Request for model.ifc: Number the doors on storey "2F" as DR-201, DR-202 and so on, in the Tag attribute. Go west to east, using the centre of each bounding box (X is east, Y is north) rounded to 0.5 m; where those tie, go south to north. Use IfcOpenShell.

First a look at what the model holds.

```python
import ifcopenshell
import ifcopenshell.util.element
import ifcopenshell.util.placement

model = ifcopenshell.open("model.ifc")
print(model.schema)
storey = next(s for s in model.by_type("IfcBuildingStorey") if s.Name == "2F")
doors = [e for e in ifcopenshell.util.element.get_decomposition(storey) if e.is_a("IfcDoor")]
for e in sorted(doors, key=lambda e: e.id()):
    origin = ifcopenshell.util.placement.get_local_placement(e.ObjectPlacement)[:3, 3]
    print(e.id(), e.Tag, e.Name, origin.round(2) + 0.0, sep=" | ")
```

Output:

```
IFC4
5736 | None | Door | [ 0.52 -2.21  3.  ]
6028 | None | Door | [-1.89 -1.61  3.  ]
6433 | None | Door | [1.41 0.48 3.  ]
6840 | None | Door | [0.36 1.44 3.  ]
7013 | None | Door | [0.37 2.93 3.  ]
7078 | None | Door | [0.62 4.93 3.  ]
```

```python
import ifcopenshell
import ifcopenshell.geom
import ifcopenshell.util.element
import ifcopenshell.util.shape

model = ifcopenshell.open("model.ifc")
settings = ifcopenshell.geom.settings()
settings.set("use-world-coords", True)


def centre(element):
    shape = ifcopenshell.geom.create_shape(settings, element)
    return ifcopenshell.util.shape.get_bbox_centroid(shape.geometry)


storey = next(s for s in model.by_type("IfcBuildingStorey") if s.Name == "2F")
doors = [e for e in ifcopenshell.util.element.get_decomposition(storey) if e.is_a("IfcDoor")]

# Insertion points can sit at a corner or the storey origin, so sort by the geometry (in metres).
centres = {e: centre(e) for e in doors}
doors.sort(key=lambda e: (round(centres[e][0] / 0.5), centres[e][1]))

for i, e in enumerate(doors, start=1):
    number = f"DR-2{i:02d}"
    e.Tag = number
    print(e.id(), number)

model.write("model_updated.ifc")
```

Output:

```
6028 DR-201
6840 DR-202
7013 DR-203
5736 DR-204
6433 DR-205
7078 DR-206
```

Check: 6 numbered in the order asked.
